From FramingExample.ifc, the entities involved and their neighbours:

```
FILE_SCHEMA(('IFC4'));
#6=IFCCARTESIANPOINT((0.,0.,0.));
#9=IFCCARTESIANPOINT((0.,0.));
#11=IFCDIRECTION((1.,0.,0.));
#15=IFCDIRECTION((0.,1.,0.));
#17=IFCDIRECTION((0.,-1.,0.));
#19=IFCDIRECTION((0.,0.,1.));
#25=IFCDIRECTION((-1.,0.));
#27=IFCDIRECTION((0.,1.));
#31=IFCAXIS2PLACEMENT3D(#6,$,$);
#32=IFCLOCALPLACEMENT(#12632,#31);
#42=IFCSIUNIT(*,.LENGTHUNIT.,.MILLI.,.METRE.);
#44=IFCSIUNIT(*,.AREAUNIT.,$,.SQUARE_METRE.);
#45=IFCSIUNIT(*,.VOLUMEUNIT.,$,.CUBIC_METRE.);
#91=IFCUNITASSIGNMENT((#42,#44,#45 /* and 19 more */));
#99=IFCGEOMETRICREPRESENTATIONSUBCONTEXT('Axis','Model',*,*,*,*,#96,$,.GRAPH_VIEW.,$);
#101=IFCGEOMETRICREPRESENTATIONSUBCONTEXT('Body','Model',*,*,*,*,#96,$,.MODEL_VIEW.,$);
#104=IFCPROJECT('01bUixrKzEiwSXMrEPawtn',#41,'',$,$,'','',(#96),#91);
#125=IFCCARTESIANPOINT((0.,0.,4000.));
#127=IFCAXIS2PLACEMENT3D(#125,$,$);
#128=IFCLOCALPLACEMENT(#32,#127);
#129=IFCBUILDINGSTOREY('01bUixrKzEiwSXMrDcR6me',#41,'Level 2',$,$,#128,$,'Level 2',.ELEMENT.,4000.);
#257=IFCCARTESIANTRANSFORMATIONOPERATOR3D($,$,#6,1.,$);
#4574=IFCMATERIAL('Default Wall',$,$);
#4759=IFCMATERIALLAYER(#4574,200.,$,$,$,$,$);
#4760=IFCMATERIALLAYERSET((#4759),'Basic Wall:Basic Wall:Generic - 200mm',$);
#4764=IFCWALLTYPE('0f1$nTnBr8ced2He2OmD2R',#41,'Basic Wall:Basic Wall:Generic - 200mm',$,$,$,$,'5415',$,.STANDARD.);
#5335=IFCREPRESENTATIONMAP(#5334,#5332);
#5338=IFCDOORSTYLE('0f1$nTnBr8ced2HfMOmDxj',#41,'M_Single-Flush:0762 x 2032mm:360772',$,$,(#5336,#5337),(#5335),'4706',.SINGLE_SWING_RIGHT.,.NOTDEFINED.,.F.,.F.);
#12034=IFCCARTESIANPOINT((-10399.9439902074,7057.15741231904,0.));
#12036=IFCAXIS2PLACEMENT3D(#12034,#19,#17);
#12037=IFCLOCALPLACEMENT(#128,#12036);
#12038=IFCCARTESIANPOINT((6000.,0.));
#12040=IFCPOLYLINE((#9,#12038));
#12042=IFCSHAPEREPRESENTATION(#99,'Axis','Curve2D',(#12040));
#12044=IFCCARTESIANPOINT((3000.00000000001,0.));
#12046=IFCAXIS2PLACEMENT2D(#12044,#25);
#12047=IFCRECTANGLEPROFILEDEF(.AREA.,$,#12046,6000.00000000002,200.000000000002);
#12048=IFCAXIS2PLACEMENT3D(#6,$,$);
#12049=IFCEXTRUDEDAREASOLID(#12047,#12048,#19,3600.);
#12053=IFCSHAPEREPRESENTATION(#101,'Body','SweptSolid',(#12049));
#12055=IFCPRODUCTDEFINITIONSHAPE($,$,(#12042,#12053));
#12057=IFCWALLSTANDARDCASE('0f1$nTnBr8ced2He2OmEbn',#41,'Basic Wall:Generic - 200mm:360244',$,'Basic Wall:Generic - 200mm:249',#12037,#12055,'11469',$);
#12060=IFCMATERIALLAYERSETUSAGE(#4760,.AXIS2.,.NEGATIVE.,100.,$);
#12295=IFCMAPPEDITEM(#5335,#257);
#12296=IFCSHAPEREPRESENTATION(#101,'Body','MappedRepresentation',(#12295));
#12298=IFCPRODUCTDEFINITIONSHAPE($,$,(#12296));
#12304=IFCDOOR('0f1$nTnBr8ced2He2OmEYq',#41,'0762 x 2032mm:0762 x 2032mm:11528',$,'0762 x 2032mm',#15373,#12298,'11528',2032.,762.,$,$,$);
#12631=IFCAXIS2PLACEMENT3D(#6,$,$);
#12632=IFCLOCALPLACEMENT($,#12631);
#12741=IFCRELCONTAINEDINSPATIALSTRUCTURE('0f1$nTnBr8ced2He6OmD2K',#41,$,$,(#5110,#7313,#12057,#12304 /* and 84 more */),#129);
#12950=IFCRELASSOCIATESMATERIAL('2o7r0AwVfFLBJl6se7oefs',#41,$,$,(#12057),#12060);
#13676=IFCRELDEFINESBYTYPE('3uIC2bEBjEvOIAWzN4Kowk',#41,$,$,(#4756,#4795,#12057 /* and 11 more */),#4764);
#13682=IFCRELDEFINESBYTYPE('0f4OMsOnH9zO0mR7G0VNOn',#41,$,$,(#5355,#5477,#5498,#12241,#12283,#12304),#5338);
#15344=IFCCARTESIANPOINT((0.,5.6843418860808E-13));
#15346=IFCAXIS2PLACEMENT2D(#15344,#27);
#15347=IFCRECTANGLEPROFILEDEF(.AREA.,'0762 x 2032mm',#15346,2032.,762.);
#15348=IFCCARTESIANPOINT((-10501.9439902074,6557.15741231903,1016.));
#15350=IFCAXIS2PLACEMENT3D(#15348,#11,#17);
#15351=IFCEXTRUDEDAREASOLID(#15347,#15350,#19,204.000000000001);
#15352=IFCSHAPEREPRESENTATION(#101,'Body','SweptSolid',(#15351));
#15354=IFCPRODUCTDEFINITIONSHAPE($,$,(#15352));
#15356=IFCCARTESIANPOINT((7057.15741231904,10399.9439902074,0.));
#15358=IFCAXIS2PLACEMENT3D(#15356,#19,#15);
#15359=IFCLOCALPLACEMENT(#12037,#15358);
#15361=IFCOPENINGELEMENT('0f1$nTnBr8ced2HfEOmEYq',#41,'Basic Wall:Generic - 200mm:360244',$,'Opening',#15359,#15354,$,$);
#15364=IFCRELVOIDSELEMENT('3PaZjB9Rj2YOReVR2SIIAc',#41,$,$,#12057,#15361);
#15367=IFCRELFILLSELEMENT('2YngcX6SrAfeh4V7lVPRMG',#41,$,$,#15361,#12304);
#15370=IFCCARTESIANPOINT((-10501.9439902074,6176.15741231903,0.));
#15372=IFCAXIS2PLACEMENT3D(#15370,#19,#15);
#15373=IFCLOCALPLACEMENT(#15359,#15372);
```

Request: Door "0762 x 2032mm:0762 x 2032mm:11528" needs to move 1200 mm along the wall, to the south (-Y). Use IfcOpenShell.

```python
import ifcopenshell
import ifcopenshell.api.geometry
import ifcopenshell.util.placement

model = ifcopenshell.open("FramingExample.ifc")

door = model.by_guid("0f1$nTnBr8ced2He2OmEYq")
opening = door.FillsVoids[0].RelatingOpeningElement
wall = opening.VoidsElements[0].RelatingBuildingElement

wall_matrix = ifcopenshell.util.placement.get_local_placement(wall.ObjectPlacement)
shift = wall_matrix[:3, 0] * 1200.0
before = ifcopenshell.util.placement.get_local_placement(door.ObjectPlacement)[:3, 3].copy()

# The door is placed relative to its opening, so it follows when the opening moves.
matrix = ifcopenshell.util.placement.get_local_placement(opening.ObjectPlacement)
matrix[:3, 3] += shift
ifcopenshell.api.geometry.edit_object_placement(
    model, product=opening, matrix=matrix, is_si=False, should_transform_children=True
)

after = ifcopenshell.util.placement.get_local_placement(door.ObjectPlacement)[:3, 3]
print("door moved by", (after - before).round(3) + 0.0)

model.write("FramingExample_v2.ifc")
```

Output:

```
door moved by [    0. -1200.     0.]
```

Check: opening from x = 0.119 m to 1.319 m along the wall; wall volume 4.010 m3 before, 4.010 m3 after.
